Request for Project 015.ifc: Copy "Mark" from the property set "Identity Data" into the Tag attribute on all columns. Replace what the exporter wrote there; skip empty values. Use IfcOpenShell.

First a look at what the model holds.

```python
import ifcopenshell
import ifcopenshell.util.element

model = ifcopenshell.open("Project 015.ifc")
print(model.schema)
columns = model.by_type("IfcColumn")
print(len(columns), "columns")
for e in columns[:8]:
    source = ifcopenshell.util.element.get_pset(e, "Identity Data", "Mark")
    target = e.Tag
    print(e.id(), repr(source), repr(target), sep=" | ")
```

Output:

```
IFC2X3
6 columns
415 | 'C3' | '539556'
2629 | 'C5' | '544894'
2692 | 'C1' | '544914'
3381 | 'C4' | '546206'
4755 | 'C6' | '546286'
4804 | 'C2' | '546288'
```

```python
import ifcopenshell
import ifcopenshell.util.element

model = ifcopenshell.open("Project 015.ifc")

count = 0
for e in model.by_type("IfcColumn"):
    value = ifcopenshell.util.element.get_pset(e, "Identity Data", "Mark")
    current = e.Tag
    if not value or not value.strip() or current == value:
        continue
    e.Tag = value
    count += 1

print(count, "columns updated")

model.write("Project 015_edited.ifc")
```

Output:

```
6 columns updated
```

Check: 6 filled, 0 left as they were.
